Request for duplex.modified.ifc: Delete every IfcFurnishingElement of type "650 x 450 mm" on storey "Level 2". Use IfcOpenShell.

First a look at what the model holds.

```python
import ifcopenshell
import ifcopenshell.util.element

model = ifcopenshell.open("duplex.modified.ifc")
print(model.schema)
storey = next(s for s in model.by_type("IfcBuildingStorey") if s.Name == "Level 2")
furniture = [e for e in ifcopenshell.util.element.get_decomposition(storey) if e.is_a("IfcFurnishingElement")]
seen = {}
for e in furniture:
    element_type = ifcopenshell.util.element.get_type(e)
    name = element_type.Name if element_type not in (None, e) else None
    seen[name] = seen.get(name, 0) + 1
for name, count in sorted(seen.items(), key=str):
    print(count, "x", name)
```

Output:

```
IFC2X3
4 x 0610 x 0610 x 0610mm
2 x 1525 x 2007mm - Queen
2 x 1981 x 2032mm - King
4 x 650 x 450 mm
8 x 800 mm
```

```python
import ifcopenshell
import ifcopenshell.api.root
import ifcopenshell.util.element

model = ifcopenshell.open("duplex.modified.ifc")

storey = next(s for s in model.by_type("IfcBuildingStorey") if s.Name == "Level 2")
furniture = [e for e in ifcopenshell.util.element.get_decomposition(storey) if e.is_a("IfcFurnishingElement")]
targets = [e for e in furniture if (t := ifcopenshell.util.element.get_type(e)) not in (None, e) and t.Name == "650 x 450 mm"]

for e in targets:
    ifcopenshell.api.root.remove_product(model, product=e)
print(len(targets), "removed")

model.write("duplex.modified_rev.ifc")
```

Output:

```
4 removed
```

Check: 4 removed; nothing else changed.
